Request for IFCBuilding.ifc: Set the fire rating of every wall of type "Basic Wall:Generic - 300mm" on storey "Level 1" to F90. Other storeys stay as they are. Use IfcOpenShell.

First a look at what the model holds.

```python
import ifcopenshell
import ifcopenshell.util.element

model = ifcopenshell.open("IFCBuilding.ifc")
print(model.schema)
storey = next(s for s in model.by_type("IfcBuildingStorey") if s.Name == "Level 1")
walls = [e for e in ifcopenshell.util.element.get_decomposition(storey) if e.is_a("IfcWall")]
seen = {}
for e in walls:
    element_type = ifcopenshell.util.element.get_type(e)
    key = (element_type.Name if element_type != e and element_type else None, ifcopenshell.util.element.get_pset(e, "Pset_WallCommon", "FireRating"))
    seen[key] = seen.get(key, 0) + 1
for (name, value), count in sorted(seen.items(), key=str):
    print(count, "x", name, "|", value)
```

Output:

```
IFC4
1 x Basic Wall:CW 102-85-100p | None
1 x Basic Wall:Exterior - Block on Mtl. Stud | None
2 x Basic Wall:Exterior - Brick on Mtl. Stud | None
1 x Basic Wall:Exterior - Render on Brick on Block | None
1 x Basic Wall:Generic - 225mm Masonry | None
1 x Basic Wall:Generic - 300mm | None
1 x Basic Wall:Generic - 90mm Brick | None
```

```python
import ifcopenshell
import ifcopenshell.api.pset
import ifcopenshell.util.element

model = ifcopenshell.open("IFCBuilding.ifc")

storey = next(s for s in model.by_type("IfcBuildingStorey") if s.Name == "Level 1")
walls = [e for e in ifcopenshell.util.element.get_decomposition(storey) if e.is_a("IfcWall")]

count = 0
for e in walls:
    element_type = ifcopenshell.util.element.get_type(e)
    if element_type in (None, e) or element_type.Name != "Basic Wall:Generic - 300mm":
        continue
    # add_pset returns the element's existing set when there is one.
    pset = ifcopenshell.api.pset.add_pset(model, product=e, name="Pset_WallCommon")
    ifcopenshell.api.pset.edit_pset(model, pset=pset, properties={"FireRating": "F90"})
    count += 1

print(count, "walls updated")

model.write("IFCBuilding_rev.ifc")
```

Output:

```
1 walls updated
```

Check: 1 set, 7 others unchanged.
